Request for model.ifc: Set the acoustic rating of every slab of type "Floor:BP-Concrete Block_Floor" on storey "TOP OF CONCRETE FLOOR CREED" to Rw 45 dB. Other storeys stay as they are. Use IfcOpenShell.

First a look at what the model holds.

```python
import ifcopenshell
import ifcopenshell.util.element

model = ifcopenshell.open("model.ifc")
print(model.schema)
storey = next(s for s in model.by_type("IfcBuildingStorey") if s.Name == "TOP OF CONCRETE FLOOR CREED")
slabs = [e for e in ifcopenshell.util.element.get_decomposition(storey) if e.is_a("IfcSlab")]
seen = {}
for e in slabs:
    element_type = ifcopenshell.util.element.get_type(e)
    key = (element_type.Name if element_type != e and element_type else None, ifcopenshell.util.element.get_pset(e, "Pset_SlabCommon", "AcousticRating"))
    seen[key] = seen.get(key, 0) + 1
for (name, value), count in sorted(seen.items(), key=str):
    print(count, "x", name, "|", value)
```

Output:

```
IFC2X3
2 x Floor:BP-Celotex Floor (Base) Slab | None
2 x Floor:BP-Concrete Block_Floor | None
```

```python
import ifcopenshell
import ifcopenshell.api.pset
import ifcopenshell.util.element

model = ifcopenshell.open("model.ifc")

storey = next(s for s in model.by_type("IfcBuildingStorey") if s.Name == "TOP OF CONCRETE FLOOR CREED")
slabs = [e for e in ifcopenshell.util.element.get_decomposition(storey) if e.is_a("IfcSlab")]

count = 0
for e in slabs:
    element_type = ifcopenshell.util.element.get_type(e)
    if element_type in (None, e) or element_type.Name != "Floor:BP-Concrete Block_Floor":
        continue
    # add_pset returns the element's existing set when there is one.
    pset = ifcopenshell.api.pset.add_pset(model, product=e, name="Pset_SlabCommon")
    ifcopenshell.api.pset.edit_pset(model, pset=pset, properties={"AcousticRating": "Rw 45 dB"})
    count += 1

print(count, "slabs updated")

model.write("model_edited.ifc")
```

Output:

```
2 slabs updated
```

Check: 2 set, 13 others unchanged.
